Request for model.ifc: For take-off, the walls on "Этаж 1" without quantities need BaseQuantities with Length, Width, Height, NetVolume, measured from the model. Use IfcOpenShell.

First a look at what the model holds.

```python
import ifcopenshell
import ifcopenshell.util.element
import ifcopenshell.util.unit

model = ifcopenshell.open("model.ifc")
print(model.schema)
for unit_type in ("LENGTHUNIT", "AREAUNIT", "VOLUMEUNIT"):
    print(unit_type, ifcopenshell.util.unit.calculate_unit_scale(model, unit_type))
storey = next(s for s in model.by_type("IfcBuildingStorey") if s.Name == "Этаж 1")
walls = [e for e in ifcopenshell.util.element.get_decomposition(storey) if e.is_a("IfcWall")]
for e in sorted(walls, key=lambda e: e.id()):
    print(e.id(), e.is_a(), e.Name, list(ifcopenshell.util.element.get_psets(e, qtos_only=True)), sep=" | ")
```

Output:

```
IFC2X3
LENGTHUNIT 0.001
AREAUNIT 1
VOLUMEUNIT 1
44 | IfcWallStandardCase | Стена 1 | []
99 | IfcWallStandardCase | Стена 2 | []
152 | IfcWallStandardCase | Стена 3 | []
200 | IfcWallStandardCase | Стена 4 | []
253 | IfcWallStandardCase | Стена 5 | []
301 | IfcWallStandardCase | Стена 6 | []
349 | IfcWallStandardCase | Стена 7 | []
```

```python
import ifcopenshell
import ifcopenshell.api.pset
import ifcopenshell.geom
import ifcopenshell.util.element
import ifcopenshell.util.shape
import ifcopenshell.util.unit

model = ifcopenshell.open("model.ifc")
unit_scale = ifcopenshell.util.unit.calculate_unit_scale(model)
volume_scale = ifcopenshell.util.unit.calculate_unit_scale(model, "VOLUMEUNIT")
settings = ifcopenshell.geom.settings()

storey = next(s for s in model.by_type("IfcBuildingStorey") if s.Name == "Этаж 1")
walls = [e for e in ifcopenshell.util.element.get_decomposition(storey) if e.is_a("IfcWall")]

for e in sorted(walls, key=lambda e: e.id()):
    if ifcopenshell.util.element.get_psets(e, qtos_only=True, should_inherit=False):
        continue
    # Geometry comes back in metres, in the element's own axes.
    shape = ifcopenshell.geom.create_shape(settings, e)
    values = {
        "Length": ifcopenshell.util.shape.get_x(shape.geometry) / unit_scale,
        "Width": ifcopenshell.util.shape.get_y(shape.geometry) / unit_scale,
        "Height": ifcopenshell.util.shape.get_z(shape.geometry) / unit_scale,
        "NetVolume": ifcopenshell.util.shape.get_volume(shape.geometry) / volume_scale,
    }
    qto = ifcopenshell.api.pset.add_qto(model, product=e, name="BaseQuantities")
    ifcopenshell.api.pset.edit_qto(model, qto=qto, properties=values)
    print(e.id(), {k: round(v, 3) for k, v in values.items()})

model.write("model_rev.ifc")
```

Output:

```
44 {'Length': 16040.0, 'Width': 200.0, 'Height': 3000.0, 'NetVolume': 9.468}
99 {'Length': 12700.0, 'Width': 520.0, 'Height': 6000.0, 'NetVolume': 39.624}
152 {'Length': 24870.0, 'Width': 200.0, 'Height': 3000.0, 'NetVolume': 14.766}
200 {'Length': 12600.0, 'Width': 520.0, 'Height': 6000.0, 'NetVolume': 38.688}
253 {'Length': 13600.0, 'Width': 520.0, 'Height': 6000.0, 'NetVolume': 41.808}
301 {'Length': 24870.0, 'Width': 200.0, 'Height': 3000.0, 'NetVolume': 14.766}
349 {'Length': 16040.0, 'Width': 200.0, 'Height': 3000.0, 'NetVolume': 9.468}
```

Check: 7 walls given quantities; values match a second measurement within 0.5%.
